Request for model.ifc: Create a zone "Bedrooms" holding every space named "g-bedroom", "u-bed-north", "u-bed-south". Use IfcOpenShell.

First a look at what the model holds.

```python
import ifcopenshell

model = ifcopenshell.open("model.ifc")
print(model.schema)
seen = {}
for space in model.by_type("IfcSpace"):
    seen[space.LongName] = seen.get(space.LongName, 0) + 1
for name, count in sorted(seen.items(), key=str):
    print(count, "x", name)
print("zones:", [z.Name for z in model.by_type("IfcZone")][:20])
```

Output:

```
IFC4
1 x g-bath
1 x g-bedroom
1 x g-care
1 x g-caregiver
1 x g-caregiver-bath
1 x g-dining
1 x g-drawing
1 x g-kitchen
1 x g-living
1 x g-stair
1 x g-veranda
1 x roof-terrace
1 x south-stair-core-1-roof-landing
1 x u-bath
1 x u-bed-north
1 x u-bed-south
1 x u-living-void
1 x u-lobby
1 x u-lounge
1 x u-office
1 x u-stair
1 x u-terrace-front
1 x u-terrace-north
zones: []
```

```python
import ifcopenshell
import ifcopenshell.api.group
import ifcopenshell.api.root

model = ifcopenshell.open("model.ifc")

names = {"g-bedroom", "u-bed-north", "u-bed-south"}
spaces = [s for s in model.by_type("IfcSpace") if s.LongName in names]

zone = ifcopenshell.api.root.create_entity(model, ifc_class="IfcZone", name="Bedrooms")
ifcopenshell.api.group.assign_group(model, products=spaces, group=zone)
print(len(spaces), "spaces in", zone.Name)

model.write("model-out.ifc")
```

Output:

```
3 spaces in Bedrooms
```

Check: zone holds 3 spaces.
